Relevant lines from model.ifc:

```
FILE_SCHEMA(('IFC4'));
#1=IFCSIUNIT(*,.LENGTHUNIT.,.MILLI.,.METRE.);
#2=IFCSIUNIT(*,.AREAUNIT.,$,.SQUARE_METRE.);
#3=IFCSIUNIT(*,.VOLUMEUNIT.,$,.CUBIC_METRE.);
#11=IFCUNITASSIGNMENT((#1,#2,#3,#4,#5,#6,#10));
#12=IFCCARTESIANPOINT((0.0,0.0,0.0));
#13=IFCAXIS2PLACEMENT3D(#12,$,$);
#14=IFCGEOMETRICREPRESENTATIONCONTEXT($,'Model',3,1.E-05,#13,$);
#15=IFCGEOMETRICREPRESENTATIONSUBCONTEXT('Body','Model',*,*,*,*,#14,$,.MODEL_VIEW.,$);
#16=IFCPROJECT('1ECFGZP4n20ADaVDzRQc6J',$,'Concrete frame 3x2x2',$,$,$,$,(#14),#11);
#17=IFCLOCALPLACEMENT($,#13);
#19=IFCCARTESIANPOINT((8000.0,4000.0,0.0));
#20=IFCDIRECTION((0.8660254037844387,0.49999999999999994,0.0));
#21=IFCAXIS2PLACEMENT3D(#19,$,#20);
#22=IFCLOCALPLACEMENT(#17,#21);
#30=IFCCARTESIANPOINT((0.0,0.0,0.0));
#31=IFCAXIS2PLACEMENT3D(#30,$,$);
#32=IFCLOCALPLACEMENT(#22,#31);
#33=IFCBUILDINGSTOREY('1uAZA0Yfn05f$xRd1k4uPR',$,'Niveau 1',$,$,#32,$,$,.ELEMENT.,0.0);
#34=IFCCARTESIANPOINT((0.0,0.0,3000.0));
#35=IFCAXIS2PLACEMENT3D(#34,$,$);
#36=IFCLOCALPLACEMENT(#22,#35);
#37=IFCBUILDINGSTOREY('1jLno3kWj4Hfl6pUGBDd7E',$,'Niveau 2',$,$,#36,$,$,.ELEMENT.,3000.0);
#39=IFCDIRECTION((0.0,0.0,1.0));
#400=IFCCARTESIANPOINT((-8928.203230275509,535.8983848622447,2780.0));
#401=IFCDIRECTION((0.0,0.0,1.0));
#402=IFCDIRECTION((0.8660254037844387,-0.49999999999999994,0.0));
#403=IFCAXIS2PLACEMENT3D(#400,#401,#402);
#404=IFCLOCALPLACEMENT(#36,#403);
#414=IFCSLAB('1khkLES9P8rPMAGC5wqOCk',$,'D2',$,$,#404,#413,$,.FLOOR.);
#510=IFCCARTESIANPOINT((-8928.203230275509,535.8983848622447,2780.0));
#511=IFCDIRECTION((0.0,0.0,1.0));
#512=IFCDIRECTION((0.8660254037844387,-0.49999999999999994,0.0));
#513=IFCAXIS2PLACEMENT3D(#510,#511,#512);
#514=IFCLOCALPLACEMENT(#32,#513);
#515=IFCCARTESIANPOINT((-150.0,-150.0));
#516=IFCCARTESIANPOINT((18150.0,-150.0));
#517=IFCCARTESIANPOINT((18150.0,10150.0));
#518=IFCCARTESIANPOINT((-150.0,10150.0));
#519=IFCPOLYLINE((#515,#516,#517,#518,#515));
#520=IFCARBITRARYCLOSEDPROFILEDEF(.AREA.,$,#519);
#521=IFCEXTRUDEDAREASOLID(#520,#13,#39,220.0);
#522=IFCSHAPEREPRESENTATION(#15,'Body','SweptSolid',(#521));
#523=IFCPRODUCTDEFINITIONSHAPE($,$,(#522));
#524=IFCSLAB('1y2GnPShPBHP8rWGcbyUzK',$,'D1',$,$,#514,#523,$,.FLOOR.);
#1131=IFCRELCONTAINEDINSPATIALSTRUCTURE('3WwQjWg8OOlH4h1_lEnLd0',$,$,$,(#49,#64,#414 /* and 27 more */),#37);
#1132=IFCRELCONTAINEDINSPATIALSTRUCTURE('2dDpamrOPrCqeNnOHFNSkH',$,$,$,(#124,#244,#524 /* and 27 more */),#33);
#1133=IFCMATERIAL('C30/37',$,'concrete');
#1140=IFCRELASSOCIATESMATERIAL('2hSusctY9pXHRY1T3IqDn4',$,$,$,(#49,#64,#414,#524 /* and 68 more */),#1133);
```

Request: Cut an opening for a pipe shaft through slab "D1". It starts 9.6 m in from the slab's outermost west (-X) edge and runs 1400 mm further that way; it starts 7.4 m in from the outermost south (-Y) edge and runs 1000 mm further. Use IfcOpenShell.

```python
import numpy as np
import ifcopenshell
import ifcopenshell.api.feature
import ifcopenshell.api.geometry
import ifcopenshell.api.root
import ifcopenshell.geom
import ifcopenshell.util.placement
import ifcopenshell.util.representation
import ifcopenshell.util.shape
import ifcopenshell.util.unit

model = ifcopenshell.open("model.ifc")
unit_scale = ifcopenshell.util.unit.calculate_unit_scale(model)
settings = ifcopenshell.geom.settings()


def volume(element):
    """Net volume in cubic metres, openings subtracted."""
    shape = ifcopenshell.geom.create_shape(settings, element)
    return ifcopenshell.util.shape.get_volume(shape.geometry)


slab = model.by_guid("1y2GnPShPBHP8rWGcbyUzK")
before = volume(slab)

# Extent in the slab's own axes, in metres. The edges named are its -X and -Y sides.
slab_shape = ifcopenshell.geom.create_shape(settings, slab)
vertices = ifcopenshell.util.shape.get_vertices(slab_shape.geometry)
x_min, y_min, bottom = vertices.min(axis=0)
top = vertices[:, 2].max()

opening = ifcopenshell.api.root.create_entity(model, ifc_class="IfcOpeningElement", name="Pipe shaft opening", predefined_type="OPENING")
context = ifcopenshell.util.representation.get_context(model, "Model", "Body", "MODEL_VIEW")
width, depth = 1.4, 1
outline = [(0.0, 0.0), (width, 0.0), (width, depth), (0.0, depth), (0.0, 0.0)]
# Overshoot both faces by 50 mm so the cut is clean.
shape = ifcopenshell.api.geometry.add_slab_representation(
    model, context=context, depth=top - bottom + 0.1, polyline=outline
)
ifcopenshell.api.geometry.assign_representation(model, product=opening, representation=shape)

matrix = ifcopenshell.util.placement.get_local_placement(slab.ObjectPlacement)
matrix[:, 3] = matrix @ np.append(np.array([x_min + 9.6, y_min + 7.4, bottom - 0.05]) / unit_scale, 1.0)
ifcopenshell.api.geometry.edit_object_placement(model, product=opening, matrix=matrix, is_si=False)
ifcopenshell.api.feature.add_feature(model, feature=opening, element=slab)

after = volume(slab)

print(f"slab volume {before:.3f} -> {after:.3f} m3")

model.write("model_rev.ifc")
```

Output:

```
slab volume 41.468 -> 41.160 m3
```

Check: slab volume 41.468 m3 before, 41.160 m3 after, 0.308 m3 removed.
